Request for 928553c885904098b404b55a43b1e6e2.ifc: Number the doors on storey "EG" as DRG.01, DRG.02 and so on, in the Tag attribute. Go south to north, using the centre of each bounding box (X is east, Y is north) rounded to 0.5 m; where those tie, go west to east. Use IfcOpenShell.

First a look at what the model holds.

```python
import ifcopenshell
import ifcopenshell.util.element
import ifcopenshell.util.placement

model = ifcopenshell.open("928553c885904098b404b55a43b1e6e2.ifc")
print(model.schema)
storey = next(s for s in model.by_type("IfcBuildingStorey") if s.Name == "EG")
doors = [e for e in ifcopenshell.util.element.get_decomposition(storey) if e.is_a("IfcDoor")]
for e in sorted(doors, key=lambda e: e.id()):
    origin = ifcopenshell.util.placement.get_local_placement(e.ObjectPlacement)[:3, 3]
    print(e.id(), e.Tag, e.Name, origin.round(2) + 0.0, sep=" | ")
```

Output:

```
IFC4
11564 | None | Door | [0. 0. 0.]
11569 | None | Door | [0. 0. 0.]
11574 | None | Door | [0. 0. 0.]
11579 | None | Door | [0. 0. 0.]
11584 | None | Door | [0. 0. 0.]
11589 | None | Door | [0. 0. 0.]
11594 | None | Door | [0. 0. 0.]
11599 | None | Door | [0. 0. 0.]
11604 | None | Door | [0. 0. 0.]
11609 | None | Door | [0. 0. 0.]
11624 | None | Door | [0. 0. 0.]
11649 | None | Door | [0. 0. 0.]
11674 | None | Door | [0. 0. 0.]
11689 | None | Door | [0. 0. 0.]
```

```python
import ifcopenshell
import ifcopenshell.geom
import ifcopenshell.util.element
import ifcopenshell.util.shape

model = ifcopenshell.open("928553c885904098b404b55a43b1e6e2.ifc")
settings = ifcopenshell.geom.settings()
settings.set("use-world-coords", True)


def centre(element):
    shape = ifcopenshell.geom.create_shape(settings, element)
    return ifcopenshell.util.shape.get_bbox_centroid(shape.geometry)


storey = next(s for s in model.by_type("IfcBuildingStorey") if s.Name == "EG")
doors = [e for e in ifcopenshell.util.element.get_decomposition(storey) if e.is_a("IfcDoor")]

# Insertion points can sit at a corner or the storey origin, so sort by the geometry (in metres).
centres = {e: centre(e) for e in doors}
doors.sort(key=lambda e: (round(centres[e][1] / 0.5), centres[e][0]))

for i, e in enumerate(doors, start=1):
    number = f"DRG.{i:02d}"
    e.Tag = number
    print(e.id(), number)

model.write("928553c885904098b404b55a43b1e6e2_updated.ifc")
```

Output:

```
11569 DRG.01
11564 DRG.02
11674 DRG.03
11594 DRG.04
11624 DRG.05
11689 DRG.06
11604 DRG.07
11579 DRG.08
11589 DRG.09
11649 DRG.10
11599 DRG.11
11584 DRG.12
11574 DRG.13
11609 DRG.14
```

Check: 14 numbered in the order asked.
